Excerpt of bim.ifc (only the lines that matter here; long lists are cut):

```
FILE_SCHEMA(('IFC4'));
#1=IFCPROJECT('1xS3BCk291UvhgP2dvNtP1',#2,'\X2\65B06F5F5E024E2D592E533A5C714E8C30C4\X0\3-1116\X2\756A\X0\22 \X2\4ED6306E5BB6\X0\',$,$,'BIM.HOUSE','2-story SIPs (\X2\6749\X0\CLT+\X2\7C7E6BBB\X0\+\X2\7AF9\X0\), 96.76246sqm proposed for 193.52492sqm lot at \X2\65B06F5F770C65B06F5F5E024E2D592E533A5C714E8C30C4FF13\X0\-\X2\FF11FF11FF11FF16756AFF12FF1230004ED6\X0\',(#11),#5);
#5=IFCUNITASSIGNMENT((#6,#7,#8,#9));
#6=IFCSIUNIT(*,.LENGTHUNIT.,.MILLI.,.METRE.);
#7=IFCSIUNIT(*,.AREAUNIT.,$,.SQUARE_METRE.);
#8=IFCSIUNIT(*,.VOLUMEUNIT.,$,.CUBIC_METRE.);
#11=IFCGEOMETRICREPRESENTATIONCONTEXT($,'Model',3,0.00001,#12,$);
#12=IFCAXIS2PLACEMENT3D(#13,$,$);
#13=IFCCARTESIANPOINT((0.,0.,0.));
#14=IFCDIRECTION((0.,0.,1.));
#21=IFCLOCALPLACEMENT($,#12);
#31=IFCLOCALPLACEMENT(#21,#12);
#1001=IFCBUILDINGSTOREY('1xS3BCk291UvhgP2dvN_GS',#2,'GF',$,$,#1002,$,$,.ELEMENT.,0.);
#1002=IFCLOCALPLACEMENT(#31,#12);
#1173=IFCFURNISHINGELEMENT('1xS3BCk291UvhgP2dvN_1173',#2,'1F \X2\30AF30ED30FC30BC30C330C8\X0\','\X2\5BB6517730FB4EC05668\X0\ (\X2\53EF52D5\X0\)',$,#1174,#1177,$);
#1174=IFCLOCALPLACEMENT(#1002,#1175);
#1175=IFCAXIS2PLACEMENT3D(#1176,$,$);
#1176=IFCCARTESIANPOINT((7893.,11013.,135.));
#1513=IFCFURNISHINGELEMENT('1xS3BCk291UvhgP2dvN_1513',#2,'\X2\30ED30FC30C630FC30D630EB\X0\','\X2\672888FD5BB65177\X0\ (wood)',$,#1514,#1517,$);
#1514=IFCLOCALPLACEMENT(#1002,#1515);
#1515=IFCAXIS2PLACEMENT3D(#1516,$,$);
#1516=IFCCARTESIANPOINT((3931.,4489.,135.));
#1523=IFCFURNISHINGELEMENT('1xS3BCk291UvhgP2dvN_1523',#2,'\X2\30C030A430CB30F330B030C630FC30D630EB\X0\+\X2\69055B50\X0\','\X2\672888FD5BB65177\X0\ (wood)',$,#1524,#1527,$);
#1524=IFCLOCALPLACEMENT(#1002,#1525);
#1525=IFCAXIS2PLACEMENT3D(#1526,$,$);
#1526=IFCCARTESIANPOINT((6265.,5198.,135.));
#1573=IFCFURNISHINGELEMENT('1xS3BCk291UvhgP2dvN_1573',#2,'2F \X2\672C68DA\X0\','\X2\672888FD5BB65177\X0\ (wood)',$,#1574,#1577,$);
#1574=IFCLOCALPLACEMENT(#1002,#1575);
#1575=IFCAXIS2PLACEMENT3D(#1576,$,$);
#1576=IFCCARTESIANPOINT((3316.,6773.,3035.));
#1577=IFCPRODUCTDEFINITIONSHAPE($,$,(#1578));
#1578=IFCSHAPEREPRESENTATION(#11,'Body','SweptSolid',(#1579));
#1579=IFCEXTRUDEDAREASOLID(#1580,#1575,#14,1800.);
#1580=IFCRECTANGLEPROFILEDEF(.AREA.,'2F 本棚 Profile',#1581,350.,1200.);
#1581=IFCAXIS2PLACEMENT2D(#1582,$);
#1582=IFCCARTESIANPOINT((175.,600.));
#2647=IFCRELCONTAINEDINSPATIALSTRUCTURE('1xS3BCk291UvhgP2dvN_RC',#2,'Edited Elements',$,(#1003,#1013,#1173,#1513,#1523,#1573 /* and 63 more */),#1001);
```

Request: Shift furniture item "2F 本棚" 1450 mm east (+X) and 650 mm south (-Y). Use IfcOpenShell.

```python
import ifcopenshell
import ifcopenshell.api.geometry
import ifcopenshell.util.placement
import ifcopenshell.util.unit

model = ifcopenshell.open("bim.ifc")
unit_scale = ifcopenshell.util.unit.calculate_unit_scale(model)

item = model.by_guid("1xS3BCk291UvhgP2dvN_1573")
matrix = ifcopenshell.util.placement.get_local_placement(item.ObjectPlacement)
matrix[0, 3] += 1.45 / unit_scale
matrix[1, 3] -= 0.65 / unit_scale
ifcopenshell.api.geometry.edit_object_placement(model, product=item, matrix=matrix, is_si=False)

print(ifcopenshell.util.placement.get_local_placement(item.ObjectPlacement).round(3) + 0.0)

model.write("bim_updated.ifc")
```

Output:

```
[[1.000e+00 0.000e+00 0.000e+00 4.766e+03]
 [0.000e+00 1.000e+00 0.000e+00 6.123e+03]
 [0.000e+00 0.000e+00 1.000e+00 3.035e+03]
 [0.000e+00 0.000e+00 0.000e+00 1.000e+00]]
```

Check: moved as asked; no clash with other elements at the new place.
